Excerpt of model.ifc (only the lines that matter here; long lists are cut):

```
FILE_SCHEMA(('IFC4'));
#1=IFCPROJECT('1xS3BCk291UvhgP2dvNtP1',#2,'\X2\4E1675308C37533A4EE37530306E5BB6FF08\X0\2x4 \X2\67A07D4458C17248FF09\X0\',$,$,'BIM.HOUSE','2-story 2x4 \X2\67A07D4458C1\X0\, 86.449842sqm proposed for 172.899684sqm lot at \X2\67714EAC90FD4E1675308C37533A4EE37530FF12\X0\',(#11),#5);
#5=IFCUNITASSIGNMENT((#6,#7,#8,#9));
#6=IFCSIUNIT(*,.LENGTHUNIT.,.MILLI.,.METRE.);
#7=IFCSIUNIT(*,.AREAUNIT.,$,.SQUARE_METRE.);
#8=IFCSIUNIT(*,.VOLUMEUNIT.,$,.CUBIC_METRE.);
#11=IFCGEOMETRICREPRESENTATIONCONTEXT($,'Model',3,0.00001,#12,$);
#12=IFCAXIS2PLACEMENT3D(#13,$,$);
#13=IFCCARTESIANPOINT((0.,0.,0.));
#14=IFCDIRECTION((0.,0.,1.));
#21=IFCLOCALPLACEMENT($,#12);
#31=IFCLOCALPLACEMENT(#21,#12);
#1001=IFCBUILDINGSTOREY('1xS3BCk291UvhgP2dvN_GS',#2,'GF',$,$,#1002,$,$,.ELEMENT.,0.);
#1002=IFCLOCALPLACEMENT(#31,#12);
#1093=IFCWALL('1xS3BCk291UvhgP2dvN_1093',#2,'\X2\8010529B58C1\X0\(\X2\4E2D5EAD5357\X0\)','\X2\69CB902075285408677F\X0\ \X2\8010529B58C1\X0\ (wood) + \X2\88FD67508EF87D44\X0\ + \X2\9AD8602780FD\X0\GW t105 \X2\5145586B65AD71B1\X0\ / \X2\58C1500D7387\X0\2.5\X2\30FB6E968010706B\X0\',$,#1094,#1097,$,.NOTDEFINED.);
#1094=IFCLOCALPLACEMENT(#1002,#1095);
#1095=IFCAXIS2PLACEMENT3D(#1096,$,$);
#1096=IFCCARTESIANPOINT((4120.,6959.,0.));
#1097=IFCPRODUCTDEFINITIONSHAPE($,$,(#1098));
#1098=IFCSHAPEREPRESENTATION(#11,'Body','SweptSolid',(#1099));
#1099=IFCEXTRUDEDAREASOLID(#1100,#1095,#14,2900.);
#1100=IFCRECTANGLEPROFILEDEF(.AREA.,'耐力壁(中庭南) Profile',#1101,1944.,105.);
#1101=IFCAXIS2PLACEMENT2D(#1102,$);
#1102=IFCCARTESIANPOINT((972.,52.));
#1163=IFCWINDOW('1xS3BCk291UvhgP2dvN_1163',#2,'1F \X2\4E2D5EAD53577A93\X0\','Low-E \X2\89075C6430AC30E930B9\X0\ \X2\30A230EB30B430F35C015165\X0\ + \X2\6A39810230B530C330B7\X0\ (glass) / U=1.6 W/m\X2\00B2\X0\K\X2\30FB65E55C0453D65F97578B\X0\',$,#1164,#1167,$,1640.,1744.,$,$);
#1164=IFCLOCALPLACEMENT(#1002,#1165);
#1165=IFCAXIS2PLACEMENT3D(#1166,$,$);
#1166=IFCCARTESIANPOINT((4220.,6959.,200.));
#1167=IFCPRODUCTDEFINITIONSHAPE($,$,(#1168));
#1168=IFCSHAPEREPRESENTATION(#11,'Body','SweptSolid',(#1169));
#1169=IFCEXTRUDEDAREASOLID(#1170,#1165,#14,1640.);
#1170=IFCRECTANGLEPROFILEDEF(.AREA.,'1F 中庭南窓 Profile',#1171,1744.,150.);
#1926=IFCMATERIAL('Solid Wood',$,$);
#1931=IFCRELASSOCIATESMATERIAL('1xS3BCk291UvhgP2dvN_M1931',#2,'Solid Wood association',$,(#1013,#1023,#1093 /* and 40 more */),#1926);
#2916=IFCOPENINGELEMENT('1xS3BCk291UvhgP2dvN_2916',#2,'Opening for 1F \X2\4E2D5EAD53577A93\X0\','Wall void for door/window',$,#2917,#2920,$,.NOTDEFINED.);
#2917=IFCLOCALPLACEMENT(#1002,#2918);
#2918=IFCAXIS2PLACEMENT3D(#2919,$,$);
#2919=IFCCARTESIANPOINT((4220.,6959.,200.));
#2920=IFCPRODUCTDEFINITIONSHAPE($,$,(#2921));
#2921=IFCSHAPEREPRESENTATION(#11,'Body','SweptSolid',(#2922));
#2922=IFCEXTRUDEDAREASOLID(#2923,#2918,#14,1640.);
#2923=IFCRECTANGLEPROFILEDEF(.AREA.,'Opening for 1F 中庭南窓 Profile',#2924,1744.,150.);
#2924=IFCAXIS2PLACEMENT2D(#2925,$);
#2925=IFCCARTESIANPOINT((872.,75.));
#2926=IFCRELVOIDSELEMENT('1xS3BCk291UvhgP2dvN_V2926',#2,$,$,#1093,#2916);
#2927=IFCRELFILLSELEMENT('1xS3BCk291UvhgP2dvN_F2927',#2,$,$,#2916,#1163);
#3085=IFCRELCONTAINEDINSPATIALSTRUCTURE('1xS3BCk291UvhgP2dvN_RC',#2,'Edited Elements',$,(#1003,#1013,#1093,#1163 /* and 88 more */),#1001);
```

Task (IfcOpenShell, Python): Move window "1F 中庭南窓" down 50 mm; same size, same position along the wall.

```python
import numpy as np
import ifcopenshell
import ifcopenshell.api.geometry
import ifcopenshell.util.placement
import ifcopenshell.util.unit

model = ifcopenshell.open("model.ifc")
unit_scale = ifcopenshell.util.unit.calculate_unit_scale(model)

window = model.by_guid("1xS3BCk291UvhgP2dvN_1163")
opening = window.FillsVoids[0].RelatingOpeningElement
dz = -0.05 / unit_scale

shift = np.array([0.0, 0.0, dz])
# The window is not placed relative to its opening, so move both.
for product in (opening, window):
    matrix = ifcopenshell.util.placement.get_local_placement(product.ObjectPlacement)
    matrix[:3, 3] += shift
    ifcopenshell.api.geometry.edit_object_placement(model, product=product, matrix=matrix, is_si=False)

print(f"moved by {dz * unit_scale:+.3f} m")

model.write("model-out.ifc")
```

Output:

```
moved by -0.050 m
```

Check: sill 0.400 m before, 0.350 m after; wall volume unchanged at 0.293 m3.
